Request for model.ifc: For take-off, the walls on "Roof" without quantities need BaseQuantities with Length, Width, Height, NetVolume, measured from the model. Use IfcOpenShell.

First a look at what the model holds.

```python
import ifcopenshell
import ifcopenshell.util.element
import ifcopenshell.util.unit

model = ifcopenshell.open("model.ifc")
print(model.schema)
for unit_type in ("LENGTHUNIT", "AREAUNIT", "VOLUMEUNIT"):
    print(unit_type, ifcopenshell.util.unit.calculate_unit_scale(model, unit_type))
storey = next(s for s in model.by_type("IfcBuildingStorey") if s.Name == "Roof")
walls = [e for e in ifcopenshell.util.element.get_decomposition(storey) if e.is_a("IfcWall")]
for e in sorted(walls, key=lambda e: e.id()):
    print(e.id(), e.is_a(), e.Name, list(ifcopenshell.util.element.get_psets(e, qtos_only=True)), sep=" | ")
```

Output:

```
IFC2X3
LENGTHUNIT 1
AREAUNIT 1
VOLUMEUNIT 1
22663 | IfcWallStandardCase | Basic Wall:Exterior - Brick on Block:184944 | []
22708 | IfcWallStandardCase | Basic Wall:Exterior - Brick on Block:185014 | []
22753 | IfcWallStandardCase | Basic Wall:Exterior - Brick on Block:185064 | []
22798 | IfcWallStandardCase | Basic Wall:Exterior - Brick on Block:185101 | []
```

```python
import ifcopenshell
import ifcopenshell.api.pset
import ifcopenshell.geom
import ifcopenshell.util.element
import ifcopenshell.util.shape
import ifcopenshell.util.unit

model = ifcopenshell.open("model.ifc")
unit_scale = ifcopenshell.util.unit.calculate_unit_scale(model)
volume_scale = ifcopenshell.util.unit.calculate_unit_scale(model, "VOLUMEUNIT")
settings = ifcopenshell.geom.settings()

storey = next(s for s in model.by_type("IfcBuildingStorey") if s.Name == "Roof")
walls = [e for e in ifcopenshell.util.element.get_decomposition(storey) if e.is_a("IfcWall")]

for e in sorted(walls, key=lambda e: e.id()):
    if ifcopenshell.util.element.get_psets(e, qtos_only=True, should_inherit=False):
        continue
    # Geometry comes back in metres, in the element's own axes.
    shape = ifcopenshell.geom.create_shape(settings, e)
    values = {
        "Length": ifcopenshell.util.shape.get_x(shape.geometry) / unit_scale,
        "Width": ifcopenshell.util.shape.get_y(shape.geometry) / unit_scale,
        "Height": ifcopenshell.util.shape.get_z(shape.geometry) / unit_scale,
        "NetVolume": ifcopenshell.util.shape.get_volume(shape.geometry) / volume_scale,
    }
    qto = ifcopenshell.api.pset.add_qto(model, product=e, name="BaseQuantities")
    ifcopenshell.api.pset.edit_qto(model, qto=qto, properties=values)
    print(e.id(), {k: round(v, 3) for k, v in values.items()})

model.write("model_updated.ifc")
```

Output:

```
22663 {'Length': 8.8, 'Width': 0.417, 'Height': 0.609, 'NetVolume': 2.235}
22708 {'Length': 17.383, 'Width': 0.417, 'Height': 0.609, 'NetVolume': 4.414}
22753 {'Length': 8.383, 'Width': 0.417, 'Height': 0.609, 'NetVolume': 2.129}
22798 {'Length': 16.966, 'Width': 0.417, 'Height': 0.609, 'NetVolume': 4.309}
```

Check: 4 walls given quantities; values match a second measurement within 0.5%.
